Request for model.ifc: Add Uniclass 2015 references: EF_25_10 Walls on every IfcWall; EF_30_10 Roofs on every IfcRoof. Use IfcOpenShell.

First a look at what the model holds.

```python
import ifcopenshell

model = ifcopenshell.open("model.ifc")
print(model.schema)
print("classifications:", [c.Name for c in model.by_type("IfcClassification")])
for ifc_class in ("IfcDoor", "IfcRoof", "IfcStair", "IfcWall", "IfcWindow"):
    print(ifc_class, len(model.by_type(ifc_class)))
```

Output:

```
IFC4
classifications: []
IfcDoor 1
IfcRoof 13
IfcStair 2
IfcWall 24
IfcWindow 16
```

```python
import ifcopenshell
import ifcopenshell.api.classification

model = ifcopenshell.open("model.ifc")

system = ifcopenshell.api.classification.add_classification(model, classification="Uniclass 2015")

codes = {
    "IfcWall": ("EF_25_10", "Walls"),
    "IfcRoof": ("EF_30_10", "Roofs"),
}
for ifc_class, (code, name) in codes.items():
    products = model.by_type(ifc_class)
    ifcopenshell.api.classification.add_reference(
        model, products=products, classification=system, identification=code, name=name
    )
    print(code, len(products))

model.write("model_edited.ifc")
```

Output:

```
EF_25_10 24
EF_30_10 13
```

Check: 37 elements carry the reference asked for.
